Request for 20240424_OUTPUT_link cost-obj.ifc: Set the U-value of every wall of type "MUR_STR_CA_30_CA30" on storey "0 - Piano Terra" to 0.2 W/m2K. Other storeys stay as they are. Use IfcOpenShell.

First a look at what the model holds.

```python
import ifcopenshell
import ifcopenshell.util.element

model = ifcopenshell.open("20240424_OUTPUT_link cost-obj.ifc")
print(model.schema)
storey = next(s for s in model.by_type("IfcBuildingStorey") if s.Name == "0 - Piano Terra")
walls = [e for e in ifcopenshell.util.element.get_decomposition(storey) if e.is_a("IfcWall")]
seen = {}
for e in walls:
    element_type = ifcopenshell.util.element.get_type(e)
    key = (element_type.Name if element_type != e and element_type else None, ifcopenshell.util.element.get_pset(e, "Pset_WallCommon", "ThermalTransmittance"))
    seen[key] = seen.get(key, 0) + 1
for (name, value), count in sorted(seen.items(), key=str):
    print(count, "x", name, "|", value)
```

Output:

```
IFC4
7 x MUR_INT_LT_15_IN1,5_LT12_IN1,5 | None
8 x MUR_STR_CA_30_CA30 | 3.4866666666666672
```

```python
import ifcopenshell
import ifcopenshell.api.pset
import ifcopenshell.util.element

model = ifcopenshell.open("20240424_OUTPUT_link cost-obj.ifc")

storey = next(s for s in model.by_type("IfcBuildingStorey") if s.Name == "0 - Piano Terra")
walls = [e for e in ifcopenshell.util.element.get_decomposition(storey) if e.is_a("IfcWall")]

count = 0
for e in walls:
    element_type = ifcopenshell.util.element.get_type(e)
    if element_type in (None, e) or element_type.Name != "MUR_STR_CA_30_CA30":
        continue
    # add_pset returns the element's existing set when there is one.
    pset = ifcopenshell.api.pset.add_pset(model, product=e, name="Pset_WallCommon")
    ifcopenshell.api.pset.edit_pset(model, pset=pset, properties={"ThermalTransmittance": 0.2})
    count += 1

print(count, "walls updated")

model.write("20240424_OUTPUT_link cost-obj_v2.ifc")
```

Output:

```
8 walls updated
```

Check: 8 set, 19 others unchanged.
